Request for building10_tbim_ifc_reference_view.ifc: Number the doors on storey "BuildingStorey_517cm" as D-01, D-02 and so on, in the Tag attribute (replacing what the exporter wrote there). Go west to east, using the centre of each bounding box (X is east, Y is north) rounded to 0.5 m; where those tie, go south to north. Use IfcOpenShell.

First a look at what the model holds.

```python
import ifcopenshell
import ifcopenshell.util.element
import ifcopenshell.util.placement

model = ifcopenshell.open("building10_tbim_ifc_reference_view.ifc")
print(model.schema)
storey = next(s for s in model.by_type("IfcBuildingStorey") if s.Name == "BuildingStorey_517cm")
doors = [e for e in ifcopenshell.util.element.get_decomposition(storey) if e.is_a("IfcDoor")]
for e in sorted(doors, key=lambda e: e.id()):
    origin = ifcopenshell.util.placement.get_local_placement(e.ObjectPlacement)[:3, 3]
    print(e.id(), e.Tag, e.Name, origin.round(2) + 0.0, sep=" | ")
```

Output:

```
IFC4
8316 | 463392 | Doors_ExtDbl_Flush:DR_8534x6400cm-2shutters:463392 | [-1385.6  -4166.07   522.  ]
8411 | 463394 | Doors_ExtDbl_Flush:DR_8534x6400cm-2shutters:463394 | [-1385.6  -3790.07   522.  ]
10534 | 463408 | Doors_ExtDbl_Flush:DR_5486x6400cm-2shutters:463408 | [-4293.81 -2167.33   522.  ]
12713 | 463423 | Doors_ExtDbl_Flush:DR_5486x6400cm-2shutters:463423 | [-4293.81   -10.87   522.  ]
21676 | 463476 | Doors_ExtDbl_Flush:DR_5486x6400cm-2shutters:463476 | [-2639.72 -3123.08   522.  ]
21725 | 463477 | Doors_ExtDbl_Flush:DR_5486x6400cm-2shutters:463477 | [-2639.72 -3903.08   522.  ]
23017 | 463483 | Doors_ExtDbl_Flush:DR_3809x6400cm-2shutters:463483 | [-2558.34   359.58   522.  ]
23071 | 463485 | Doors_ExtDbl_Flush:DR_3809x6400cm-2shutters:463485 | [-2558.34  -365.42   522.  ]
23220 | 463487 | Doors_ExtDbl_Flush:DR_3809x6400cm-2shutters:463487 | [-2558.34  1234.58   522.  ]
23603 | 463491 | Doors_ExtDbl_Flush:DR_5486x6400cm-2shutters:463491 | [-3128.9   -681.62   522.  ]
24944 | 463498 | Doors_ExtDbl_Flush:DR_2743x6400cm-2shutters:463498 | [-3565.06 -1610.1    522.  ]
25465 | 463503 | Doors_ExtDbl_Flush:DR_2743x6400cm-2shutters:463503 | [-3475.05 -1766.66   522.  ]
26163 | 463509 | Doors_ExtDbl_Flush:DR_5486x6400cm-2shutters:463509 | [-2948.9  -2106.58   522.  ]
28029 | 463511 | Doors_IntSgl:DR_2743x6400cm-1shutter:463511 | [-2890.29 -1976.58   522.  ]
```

```python
import ifcopenshell
import ifcopenshell.geom
import ifcopenshell.util.element
import ifcopenshell.util.shape

model = ifcopenshell.open("building10_tbim_ifc_reference_view.ifc")
settings = ifcopenshell.geom.settings()
settings.set("use-world-coords", True)


def centre(element):
    shape = ifcopenshell.geom.create_shape(settings, element)
    return ifcopenshell.util.shape.get_bbox_centroid(shape.geometry)


storey = next(s for s in model.by_type("IfcBuildingStorey") if s.Name == "BuildingStorey_517cm")
doors = [e for e in ifcopenshell.util.element.get_decomposition(storey) if e.is_a("IfcDoor")]

# Insertion points can sit at a corner or the storey origin, so sort by the geometry (in metres).
centres = {e: centre(e) for e in doors}
doors.sort(key=lambda e: (round(centres[e][0] / 0.5), centres[e][1]))

for i, e in enumerate(doors, start=1):
    number = f"D-{i:02d}"
    e.Tag = number
    print(e.id(), number)

model.write("building10_tbim_ifc_reference_view_rev.ifc")
```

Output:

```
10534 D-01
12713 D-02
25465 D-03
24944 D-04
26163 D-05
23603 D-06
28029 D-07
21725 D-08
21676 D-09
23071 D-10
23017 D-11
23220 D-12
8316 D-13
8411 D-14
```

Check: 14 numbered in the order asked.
